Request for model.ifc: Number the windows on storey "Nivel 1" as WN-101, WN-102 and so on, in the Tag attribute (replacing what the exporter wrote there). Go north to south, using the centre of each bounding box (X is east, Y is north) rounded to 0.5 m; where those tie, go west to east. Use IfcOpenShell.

First a look at what the model holds.

```python
import ifcopenshell
import ifcopenshell.util.element
import ifcopenshell.util.placement

model = ifcopenshell.open("model.ifc")
print(model.schema)
storey = next(s for s in model.by_type("IfcBuildingStorey") if s.Name == "Nivel 1")
windows = [e for e in ifcopenshell.util.element.get_decomposition(storey) if e.is_a("IfcWindow")]
for e in sorted(windows, key=lambda e: e.id()):
    origin = ifcopenshell.util.placement.get_local_placement(e.ObjectPlacement)[:3, 3]
    print(e.id(), e.Tag, e.Name, origin.round(2) + 0.0, sep=" | ")
```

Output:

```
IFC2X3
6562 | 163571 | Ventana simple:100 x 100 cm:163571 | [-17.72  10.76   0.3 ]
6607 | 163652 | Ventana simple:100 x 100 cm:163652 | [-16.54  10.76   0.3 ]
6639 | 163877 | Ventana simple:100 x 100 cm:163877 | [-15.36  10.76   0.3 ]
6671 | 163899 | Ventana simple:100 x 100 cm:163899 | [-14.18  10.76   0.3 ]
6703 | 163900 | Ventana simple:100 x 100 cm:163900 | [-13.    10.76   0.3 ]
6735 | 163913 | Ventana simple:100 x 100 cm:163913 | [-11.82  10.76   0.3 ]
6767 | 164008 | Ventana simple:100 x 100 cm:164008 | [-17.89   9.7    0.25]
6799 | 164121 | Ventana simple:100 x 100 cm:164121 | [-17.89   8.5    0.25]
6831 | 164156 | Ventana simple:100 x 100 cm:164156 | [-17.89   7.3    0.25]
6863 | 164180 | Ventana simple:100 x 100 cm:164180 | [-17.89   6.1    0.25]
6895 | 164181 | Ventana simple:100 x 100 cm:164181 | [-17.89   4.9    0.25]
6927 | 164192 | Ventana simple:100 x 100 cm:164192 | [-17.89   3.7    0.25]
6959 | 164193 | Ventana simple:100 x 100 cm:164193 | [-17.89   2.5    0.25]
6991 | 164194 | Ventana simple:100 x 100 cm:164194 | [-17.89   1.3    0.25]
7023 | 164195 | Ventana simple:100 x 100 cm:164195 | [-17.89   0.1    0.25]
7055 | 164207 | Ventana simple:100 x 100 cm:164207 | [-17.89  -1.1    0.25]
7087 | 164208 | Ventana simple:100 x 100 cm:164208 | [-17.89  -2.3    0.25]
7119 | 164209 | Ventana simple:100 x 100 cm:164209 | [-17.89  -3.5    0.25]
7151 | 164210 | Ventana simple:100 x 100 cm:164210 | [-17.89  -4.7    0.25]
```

```python
import ifcopenshell
import ifcopenshell.geom
import ifcopenshell.util.element
import ifcopenshell.util.shape

model = ifcopenshell.open("model.ifc")
settings = ifcopenshell.geom.settings()
settings.set("use-world-coords", True)


def centre(element):
    shape = ifcopenshell.geom.create_shape(settings, element)
    return ifcopenshell.util.shape.get_bbox_centroid(shape.geometry)


storey = next(s for s in model.by_type("IfcBuildingStorey") if s.Name == "Nivel 1")
windows = [e for e in ifcopenshell.util.element.get_decomposition(storey) if e.is_a("IfcWindow")]

# Insertion points can sit at a corner or the storey origin, so sort by the geometry (in metres).
centres = {e: centre(e) for e in windows}
windows.sort(key=lambda e: (-round(centres[e][1] / 0.5), centres[e][0]))

for i, e in enumerate(windows, start=1):
    number = f"WN-1{i:02d}"
    e.Tag = number
    print(e.id(), number)

model.write("model_edited.ifc")
```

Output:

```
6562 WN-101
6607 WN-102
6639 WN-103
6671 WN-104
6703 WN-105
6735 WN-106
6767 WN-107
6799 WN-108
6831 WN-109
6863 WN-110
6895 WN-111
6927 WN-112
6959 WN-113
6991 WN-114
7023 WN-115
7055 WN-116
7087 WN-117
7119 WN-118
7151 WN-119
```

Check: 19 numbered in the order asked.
